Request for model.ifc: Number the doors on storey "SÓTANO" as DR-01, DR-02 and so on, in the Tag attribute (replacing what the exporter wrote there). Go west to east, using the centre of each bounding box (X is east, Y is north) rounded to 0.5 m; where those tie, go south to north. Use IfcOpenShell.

First a look at what the model holds.

```python
import ifcopenshell
import ifcopenshell.util.element
import ifcopenshell.util.placement

model = ifcopenshell.open("model.ifc")
print(model.schema)
storey = next(s for s in model.by_type("IfcBuildingStorey") if s.Name == "SÓTANO")
doors = [e for e in ifcopenshell.util.element.get_decomposition(storey) if e.is_a("IfcDoor")]
for e in sorted(doors, key=lambda e: e.id()):
    origin = ifcopenshell.util.placement.get_local_placement(e.ObjectPlacement)[:3, 3]
    print(e.id(), e.Tag, e.Name, origin.round(2) + 0.0, sep=" | ")
```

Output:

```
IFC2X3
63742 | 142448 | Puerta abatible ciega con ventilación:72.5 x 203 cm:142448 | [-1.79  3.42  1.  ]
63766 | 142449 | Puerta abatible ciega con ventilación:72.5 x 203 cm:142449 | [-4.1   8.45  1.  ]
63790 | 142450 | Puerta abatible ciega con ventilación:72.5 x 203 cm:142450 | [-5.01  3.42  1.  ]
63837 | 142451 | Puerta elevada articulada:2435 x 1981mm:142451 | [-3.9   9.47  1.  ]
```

```python
import ifcopenshell
import ifcopenshell.geom
import ifcopenshell.util.element
import ifcopenshell.util.shape

model = ifcopenshell.open("model.ifc")
settings = ifcopenshell.geom.settings()
settings.set("use-world-coords", True)


def centre(element):
    shape = ifcopenshell.geom.create_shape(settings, element)
    return ifcopenshell.util.shape.get_bbox_centroid(shape.geometry)


storey = next(s for s in model.by_type("IfcBuildingStorey") if s.Name == "SÓTANO")
doors = [e for e in ifcopenshell.util.element.get_decomposition(storey) if e.is_a("IfcDoor")]

# Insertion points can sit at a corner or the storey origin, so sort by the geometry (in metres).
centres = {e: centre(e) for e in doors}
doors.sort(key=lambda e: (round(centres[e][0] / 0.5), centres[e][1]))

for i, e in enumerate(doors, start=1):
    number = f"DR-{i:02d}"
    e.Tag = number
    print(e.id(), number)

model.write("model-out.ifc")
```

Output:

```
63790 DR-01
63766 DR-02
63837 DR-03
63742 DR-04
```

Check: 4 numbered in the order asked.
